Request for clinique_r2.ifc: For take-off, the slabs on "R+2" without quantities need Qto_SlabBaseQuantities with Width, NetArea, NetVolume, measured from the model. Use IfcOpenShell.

First a look at what the model holds.

```python
import ifcopenshell
import ifcopenshell.util.element
import ifcopenshell.util.unit

model = ifcopenshell.open("clinique_r2.ifc")
print(model.schema)
for unit_type in ("LENGTHUNIT", "AREAUNIT", "VOLUMEUNIT"):
    print(unit_type, ifcopenshell.util.unit.calculate_unit_scale(model, unit_type))
storey = next(s for s in model.by_type("IfcBuildingStorey") if s.Name == "R+2")
slabs = [e for e in ifcopenshell.util.element.get_decomposition(storey) if e.is_a("IfcSlab")]
for e in sorted(slabs, key=lambda e: e.id()):
    print(e.id(), e.is_a(), e.Name, list(ifcopenshell.util.element.get_psets(e, qtos_only=True)), sep=" | ")
```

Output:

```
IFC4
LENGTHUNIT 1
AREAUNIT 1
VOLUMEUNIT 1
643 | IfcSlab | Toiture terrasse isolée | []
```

```python
import ifcopenshell
import ifcopenshell.api.pset
import ifcopenshell.geom
import ifcopenshell.util.element
import ifcopenshell.util.shape
import ifcopenshell.util.unit

model = ifcopenshell.open("clinique_r2.ifc")
unit_scale = ifcopenshell.util.unit.calculate_unit_scale(model)
area_scale = ifcopenshell.util.unit.calculate_unit_scale(model, "AREAUNIT")
volume_scale = ifcopenshell.util.unit.calculate_unit_scale(model, "VOLUMEUNIT")
settings = ifcopenshell.geom.settings()

storey = next(s for s in model.by_type("IfcBuildingStorey") if s.Name == "R+2")
slabs = [e for e in ifcopenshell.util.element.get_decomposition(storey) if e.is_a("IfcSlab")]

for e in sorted(slabs, key=lambda e: e.id()):
    if ifcopenshell.util.element.get_psets(e, qtos_only=True, should_inherit=False):
        continue
    # Geometry comes back in metres, in the element's own axes.
    shape = ifcopenshell.geom.create_shape(settings, e)
    values = {
        "Width": ifcopenshell.util.shape.get_z(shape.geometry) / unit_scale,
        "NetArea": ifcopenshell.util.shape.get_footprint_area(shape.geometry) / area_scale,
        "NetVolume": ifcopenshell.util.shape.get_volume(shape.geometry) / volume_scale,
    }
    qto = ifcopenshell.api.pset.add_qto(model, product=e, name="Qto_SlabBaseQuantities")
    ifcopenshell.api.pset.edit_qto(model, qto=qto, properties=values)
    print(e.id(), {k: round(v, 3) for k, v in values.items()})

model.write("clinique_r2_updated.ifc")
```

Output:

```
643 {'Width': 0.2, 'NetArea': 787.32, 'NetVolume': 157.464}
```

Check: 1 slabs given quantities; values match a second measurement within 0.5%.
